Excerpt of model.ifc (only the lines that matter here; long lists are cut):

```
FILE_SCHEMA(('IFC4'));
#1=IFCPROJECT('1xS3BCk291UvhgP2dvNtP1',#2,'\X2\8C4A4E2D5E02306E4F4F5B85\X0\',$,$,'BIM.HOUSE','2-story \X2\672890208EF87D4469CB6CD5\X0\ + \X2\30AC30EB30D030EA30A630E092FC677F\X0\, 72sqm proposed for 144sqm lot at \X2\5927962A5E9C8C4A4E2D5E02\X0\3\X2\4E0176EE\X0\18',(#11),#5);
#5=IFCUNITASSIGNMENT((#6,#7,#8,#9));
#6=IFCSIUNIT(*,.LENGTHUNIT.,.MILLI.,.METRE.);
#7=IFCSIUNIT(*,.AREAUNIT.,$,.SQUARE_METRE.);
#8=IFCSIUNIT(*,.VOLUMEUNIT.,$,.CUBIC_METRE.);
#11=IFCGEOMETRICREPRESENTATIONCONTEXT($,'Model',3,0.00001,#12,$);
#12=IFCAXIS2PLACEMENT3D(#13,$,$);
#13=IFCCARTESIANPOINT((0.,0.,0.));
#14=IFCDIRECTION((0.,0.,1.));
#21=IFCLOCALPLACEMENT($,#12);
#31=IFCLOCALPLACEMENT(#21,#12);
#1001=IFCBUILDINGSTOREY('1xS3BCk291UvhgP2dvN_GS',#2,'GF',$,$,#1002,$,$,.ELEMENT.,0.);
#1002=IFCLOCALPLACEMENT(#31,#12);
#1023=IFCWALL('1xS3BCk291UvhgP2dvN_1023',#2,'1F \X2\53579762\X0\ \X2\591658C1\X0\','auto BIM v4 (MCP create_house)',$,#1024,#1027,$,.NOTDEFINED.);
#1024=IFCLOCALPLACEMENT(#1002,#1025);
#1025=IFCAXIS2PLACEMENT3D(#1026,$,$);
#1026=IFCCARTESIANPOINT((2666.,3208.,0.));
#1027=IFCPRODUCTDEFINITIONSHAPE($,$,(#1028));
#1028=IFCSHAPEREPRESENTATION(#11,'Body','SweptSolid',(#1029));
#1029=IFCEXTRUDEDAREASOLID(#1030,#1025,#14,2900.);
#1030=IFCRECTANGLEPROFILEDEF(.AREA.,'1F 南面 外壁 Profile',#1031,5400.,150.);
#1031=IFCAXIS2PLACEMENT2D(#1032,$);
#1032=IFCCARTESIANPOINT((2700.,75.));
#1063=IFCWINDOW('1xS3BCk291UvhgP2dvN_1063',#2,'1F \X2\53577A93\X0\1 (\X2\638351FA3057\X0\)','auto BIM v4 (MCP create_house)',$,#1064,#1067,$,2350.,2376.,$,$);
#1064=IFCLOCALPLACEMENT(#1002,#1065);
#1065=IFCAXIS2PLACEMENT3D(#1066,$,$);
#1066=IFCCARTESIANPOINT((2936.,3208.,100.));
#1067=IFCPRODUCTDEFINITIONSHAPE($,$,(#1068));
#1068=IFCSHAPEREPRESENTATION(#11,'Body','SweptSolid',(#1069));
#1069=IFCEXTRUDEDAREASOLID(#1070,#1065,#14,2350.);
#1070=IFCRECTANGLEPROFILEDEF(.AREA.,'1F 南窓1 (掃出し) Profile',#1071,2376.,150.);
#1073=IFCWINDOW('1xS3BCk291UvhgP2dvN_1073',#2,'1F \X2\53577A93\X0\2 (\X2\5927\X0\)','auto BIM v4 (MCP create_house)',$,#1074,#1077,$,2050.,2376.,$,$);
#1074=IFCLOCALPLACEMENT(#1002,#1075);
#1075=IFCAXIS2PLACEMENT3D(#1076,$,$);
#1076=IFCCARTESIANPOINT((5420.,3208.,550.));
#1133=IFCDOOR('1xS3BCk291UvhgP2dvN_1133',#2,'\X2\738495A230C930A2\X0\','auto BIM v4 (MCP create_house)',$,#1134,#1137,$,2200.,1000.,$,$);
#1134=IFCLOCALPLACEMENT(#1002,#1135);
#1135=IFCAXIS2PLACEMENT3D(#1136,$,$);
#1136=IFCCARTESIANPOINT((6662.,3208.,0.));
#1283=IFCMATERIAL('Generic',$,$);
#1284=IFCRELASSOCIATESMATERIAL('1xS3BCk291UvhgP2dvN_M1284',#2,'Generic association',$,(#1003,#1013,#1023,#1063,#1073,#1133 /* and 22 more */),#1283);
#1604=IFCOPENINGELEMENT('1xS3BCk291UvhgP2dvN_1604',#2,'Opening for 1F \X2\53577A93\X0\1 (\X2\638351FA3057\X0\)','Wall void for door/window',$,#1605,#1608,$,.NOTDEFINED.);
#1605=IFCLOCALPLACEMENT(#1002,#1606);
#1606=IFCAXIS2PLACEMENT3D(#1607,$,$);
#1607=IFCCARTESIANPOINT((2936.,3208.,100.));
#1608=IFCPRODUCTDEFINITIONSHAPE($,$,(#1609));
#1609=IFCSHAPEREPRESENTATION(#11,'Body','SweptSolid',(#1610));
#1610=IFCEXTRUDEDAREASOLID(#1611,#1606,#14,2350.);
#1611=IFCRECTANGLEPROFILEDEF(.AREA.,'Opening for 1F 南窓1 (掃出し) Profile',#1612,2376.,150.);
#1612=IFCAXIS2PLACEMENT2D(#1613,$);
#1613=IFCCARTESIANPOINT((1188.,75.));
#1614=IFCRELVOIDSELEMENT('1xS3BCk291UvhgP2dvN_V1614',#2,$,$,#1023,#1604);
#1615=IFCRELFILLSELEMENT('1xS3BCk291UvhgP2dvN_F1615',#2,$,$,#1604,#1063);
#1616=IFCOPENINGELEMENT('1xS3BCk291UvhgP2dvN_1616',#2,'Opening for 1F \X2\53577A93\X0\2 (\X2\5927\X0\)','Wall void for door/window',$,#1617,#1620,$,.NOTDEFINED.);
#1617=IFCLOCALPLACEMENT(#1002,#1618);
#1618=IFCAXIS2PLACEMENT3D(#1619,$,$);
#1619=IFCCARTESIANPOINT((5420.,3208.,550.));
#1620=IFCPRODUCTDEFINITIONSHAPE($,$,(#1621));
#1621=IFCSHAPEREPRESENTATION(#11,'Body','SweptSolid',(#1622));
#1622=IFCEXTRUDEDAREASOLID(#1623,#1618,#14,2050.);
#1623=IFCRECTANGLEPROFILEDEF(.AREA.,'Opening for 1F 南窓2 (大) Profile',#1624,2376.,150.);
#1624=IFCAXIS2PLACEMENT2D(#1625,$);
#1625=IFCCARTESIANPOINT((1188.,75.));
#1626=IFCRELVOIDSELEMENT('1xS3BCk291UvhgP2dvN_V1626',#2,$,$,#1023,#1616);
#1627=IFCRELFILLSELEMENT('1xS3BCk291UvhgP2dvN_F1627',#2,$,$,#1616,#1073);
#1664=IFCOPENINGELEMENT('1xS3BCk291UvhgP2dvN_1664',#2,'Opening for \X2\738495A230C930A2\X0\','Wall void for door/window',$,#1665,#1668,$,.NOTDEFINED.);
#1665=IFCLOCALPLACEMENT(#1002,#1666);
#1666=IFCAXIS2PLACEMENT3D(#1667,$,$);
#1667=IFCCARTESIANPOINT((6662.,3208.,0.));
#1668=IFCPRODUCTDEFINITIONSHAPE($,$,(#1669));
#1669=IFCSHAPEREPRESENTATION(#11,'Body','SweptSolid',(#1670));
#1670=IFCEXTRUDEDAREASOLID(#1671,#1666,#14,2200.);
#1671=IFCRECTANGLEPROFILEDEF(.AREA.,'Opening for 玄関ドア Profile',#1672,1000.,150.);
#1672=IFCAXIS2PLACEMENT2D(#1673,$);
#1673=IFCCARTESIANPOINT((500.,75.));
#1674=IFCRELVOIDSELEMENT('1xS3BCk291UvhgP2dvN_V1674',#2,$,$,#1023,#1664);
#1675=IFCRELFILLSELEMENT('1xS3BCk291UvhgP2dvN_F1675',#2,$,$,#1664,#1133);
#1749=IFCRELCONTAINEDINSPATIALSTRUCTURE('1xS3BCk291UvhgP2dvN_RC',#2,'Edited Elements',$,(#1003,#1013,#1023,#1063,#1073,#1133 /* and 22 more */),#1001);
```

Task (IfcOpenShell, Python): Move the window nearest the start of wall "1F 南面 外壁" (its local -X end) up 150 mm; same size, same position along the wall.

```python
import numpy as np
import ifcopenshell
import ifcopenshell.api.geometry
import ifcopenshell.util.placement
import ifcopenshell.util.unit

model = ifcopenshell.open("model.ifc")
unit_scale = ifcopenshell.util.unit.calculate_unit_scale(model)

window = model.by_guid("1xS3BCk291UvhgP2dvN_1063")
opening = window.FillsVoids[0].RelatingOpeningElement
dz = 150.0

shift = np.array([0.0, 0.0, dz])
# The window is not placed relative to its opening, so move both.
for product in (opening, window):
    matrix = ifcopenshell.util.placement.get_local_placement(product.ObjectPlacement)
    matrix[:3, 3] += shift
    ifcopenshell.api.geometry.edit_object_placement(model, product=product, matrix=matrix, is_si=False)

print(f"moved by {dz * unit_scale:+.3f} m")

model.write("model_edited.ifc")
```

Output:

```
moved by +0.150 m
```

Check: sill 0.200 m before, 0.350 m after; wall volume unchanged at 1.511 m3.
